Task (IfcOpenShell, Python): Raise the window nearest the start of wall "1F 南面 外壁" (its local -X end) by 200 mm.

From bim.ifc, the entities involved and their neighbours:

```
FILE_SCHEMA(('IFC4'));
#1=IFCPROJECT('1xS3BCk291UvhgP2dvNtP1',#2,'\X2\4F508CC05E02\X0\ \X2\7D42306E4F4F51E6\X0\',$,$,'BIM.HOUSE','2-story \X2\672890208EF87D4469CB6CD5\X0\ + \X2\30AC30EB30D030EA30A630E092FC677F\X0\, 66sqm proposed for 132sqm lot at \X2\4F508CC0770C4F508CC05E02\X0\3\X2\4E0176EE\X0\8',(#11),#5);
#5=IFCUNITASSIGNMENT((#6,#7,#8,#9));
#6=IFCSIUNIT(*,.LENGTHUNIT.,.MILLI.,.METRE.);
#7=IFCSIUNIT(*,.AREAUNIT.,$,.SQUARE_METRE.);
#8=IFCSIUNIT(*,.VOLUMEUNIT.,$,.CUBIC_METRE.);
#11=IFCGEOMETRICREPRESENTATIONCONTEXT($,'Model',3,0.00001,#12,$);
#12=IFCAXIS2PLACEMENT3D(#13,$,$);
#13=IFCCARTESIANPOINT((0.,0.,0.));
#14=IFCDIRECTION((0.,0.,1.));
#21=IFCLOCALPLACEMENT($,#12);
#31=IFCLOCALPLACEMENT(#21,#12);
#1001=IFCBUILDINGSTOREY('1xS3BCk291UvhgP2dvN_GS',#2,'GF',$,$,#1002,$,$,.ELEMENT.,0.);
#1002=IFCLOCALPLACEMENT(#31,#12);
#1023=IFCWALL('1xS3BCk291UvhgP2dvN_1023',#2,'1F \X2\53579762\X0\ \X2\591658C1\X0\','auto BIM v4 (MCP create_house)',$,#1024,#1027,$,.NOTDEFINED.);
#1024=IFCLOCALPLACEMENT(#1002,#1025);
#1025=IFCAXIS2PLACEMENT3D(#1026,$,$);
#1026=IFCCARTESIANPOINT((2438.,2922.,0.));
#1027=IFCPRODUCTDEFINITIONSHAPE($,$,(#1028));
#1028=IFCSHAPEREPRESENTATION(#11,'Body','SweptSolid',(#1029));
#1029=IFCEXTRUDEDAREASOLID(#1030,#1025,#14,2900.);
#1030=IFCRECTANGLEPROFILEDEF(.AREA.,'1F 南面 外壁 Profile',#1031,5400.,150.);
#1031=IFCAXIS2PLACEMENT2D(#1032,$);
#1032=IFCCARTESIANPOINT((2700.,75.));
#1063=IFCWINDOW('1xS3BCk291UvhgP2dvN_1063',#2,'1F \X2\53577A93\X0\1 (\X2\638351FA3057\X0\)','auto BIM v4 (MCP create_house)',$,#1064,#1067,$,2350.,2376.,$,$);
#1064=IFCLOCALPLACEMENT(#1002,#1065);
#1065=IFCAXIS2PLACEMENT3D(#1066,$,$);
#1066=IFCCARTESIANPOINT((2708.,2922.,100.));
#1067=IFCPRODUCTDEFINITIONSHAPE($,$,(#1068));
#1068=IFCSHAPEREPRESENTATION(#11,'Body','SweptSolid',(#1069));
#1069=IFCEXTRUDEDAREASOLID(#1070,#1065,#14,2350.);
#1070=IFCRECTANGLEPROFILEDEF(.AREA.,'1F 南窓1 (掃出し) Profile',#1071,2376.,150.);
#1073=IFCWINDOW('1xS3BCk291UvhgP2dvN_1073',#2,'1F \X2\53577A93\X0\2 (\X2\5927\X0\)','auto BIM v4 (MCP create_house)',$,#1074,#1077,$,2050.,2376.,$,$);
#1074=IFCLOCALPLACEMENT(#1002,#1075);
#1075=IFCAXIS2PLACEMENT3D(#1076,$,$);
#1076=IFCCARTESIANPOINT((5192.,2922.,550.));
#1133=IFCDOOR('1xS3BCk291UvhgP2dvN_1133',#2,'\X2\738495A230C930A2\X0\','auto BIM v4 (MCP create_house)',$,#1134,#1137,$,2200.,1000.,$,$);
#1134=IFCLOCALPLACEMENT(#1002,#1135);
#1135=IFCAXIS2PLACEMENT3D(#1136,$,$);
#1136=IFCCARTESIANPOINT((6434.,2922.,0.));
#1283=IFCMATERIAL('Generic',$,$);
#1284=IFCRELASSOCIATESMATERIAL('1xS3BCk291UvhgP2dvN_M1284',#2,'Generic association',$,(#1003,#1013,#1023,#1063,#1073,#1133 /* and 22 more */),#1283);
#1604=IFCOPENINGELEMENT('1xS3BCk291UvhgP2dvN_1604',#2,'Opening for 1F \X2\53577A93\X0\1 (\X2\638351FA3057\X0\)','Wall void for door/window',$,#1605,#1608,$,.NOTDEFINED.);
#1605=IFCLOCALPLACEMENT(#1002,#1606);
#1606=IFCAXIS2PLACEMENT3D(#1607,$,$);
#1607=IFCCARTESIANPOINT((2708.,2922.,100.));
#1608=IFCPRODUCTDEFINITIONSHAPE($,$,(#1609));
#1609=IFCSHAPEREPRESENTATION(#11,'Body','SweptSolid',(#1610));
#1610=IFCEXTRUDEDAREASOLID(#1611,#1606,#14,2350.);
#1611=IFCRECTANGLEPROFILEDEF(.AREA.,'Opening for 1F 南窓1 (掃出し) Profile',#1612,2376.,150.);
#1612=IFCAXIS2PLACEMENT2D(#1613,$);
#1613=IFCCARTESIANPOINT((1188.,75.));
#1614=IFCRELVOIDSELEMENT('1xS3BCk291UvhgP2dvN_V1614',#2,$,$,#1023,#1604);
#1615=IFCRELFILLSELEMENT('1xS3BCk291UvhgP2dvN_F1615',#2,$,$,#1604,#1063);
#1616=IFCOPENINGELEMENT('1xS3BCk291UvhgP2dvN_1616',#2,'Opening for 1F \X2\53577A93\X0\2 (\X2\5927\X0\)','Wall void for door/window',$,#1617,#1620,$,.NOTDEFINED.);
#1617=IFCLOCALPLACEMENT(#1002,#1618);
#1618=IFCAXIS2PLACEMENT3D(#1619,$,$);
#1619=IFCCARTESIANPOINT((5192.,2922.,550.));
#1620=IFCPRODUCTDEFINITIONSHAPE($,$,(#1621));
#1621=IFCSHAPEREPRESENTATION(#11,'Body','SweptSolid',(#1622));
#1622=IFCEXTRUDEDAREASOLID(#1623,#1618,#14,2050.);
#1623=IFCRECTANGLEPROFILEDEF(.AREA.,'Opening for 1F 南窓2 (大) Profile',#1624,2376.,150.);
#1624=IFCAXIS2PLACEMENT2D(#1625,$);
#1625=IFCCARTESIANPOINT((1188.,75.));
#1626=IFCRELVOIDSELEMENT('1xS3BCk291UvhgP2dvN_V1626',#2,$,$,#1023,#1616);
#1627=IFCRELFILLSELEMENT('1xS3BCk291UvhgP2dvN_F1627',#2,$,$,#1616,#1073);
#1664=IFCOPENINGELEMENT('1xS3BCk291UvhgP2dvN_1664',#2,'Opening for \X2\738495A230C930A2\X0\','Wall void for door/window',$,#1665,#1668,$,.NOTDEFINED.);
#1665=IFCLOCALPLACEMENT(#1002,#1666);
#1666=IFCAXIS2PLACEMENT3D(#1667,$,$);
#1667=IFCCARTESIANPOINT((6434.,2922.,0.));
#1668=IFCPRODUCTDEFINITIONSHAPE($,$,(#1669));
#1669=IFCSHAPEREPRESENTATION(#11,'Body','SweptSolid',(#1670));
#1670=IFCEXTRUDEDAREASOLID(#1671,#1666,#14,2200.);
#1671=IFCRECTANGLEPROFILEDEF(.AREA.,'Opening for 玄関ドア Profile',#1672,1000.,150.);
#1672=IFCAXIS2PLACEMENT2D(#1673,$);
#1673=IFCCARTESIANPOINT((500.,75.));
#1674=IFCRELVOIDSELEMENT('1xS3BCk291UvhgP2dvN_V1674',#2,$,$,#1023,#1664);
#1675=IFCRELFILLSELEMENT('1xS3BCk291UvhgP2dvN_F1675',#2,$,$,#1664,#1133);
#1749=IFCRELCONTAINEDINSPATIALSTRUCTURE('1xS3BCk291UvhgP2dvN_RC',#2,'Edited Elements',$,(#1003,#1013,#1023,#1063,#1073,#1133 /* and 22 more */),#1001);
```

```python
import numpy as np
import ifcopenshell
import ifcopenshell.api.geometry
import ifcopenshell.util.placement
import ifcopenshell.util.unit

model = ifcopenshell.open("bim.ifc")
unit_scale = ifcopenshell.util.unit.calculate_unit_scale(model)

window = model.by_guid("1xS3BCk291UvhgP2dvN_1063")
opening = window.FillsVoids[0].RelatingOpeningElement
dz = 200.0

shift = np.array([0.0, 0.0, dz])
# The window is not placed relative to its opening, so move both.
for product in (opening, window):
    matrix = ifcopenshell.util.placement.get_local_placement(product.ObjectPlacement)
    matrix[:3, 3] += shift
    ifcopenshell.api.geometry.edit_object_placement(model, product=product, matrix=matrix, is_si=False)

print(f"moved by {dz * unit_scale:+.3f} m")

model.write("bim-out.ifc")
```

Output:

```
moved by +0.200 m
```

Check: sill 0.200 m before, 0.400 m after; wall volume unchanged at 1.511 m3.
